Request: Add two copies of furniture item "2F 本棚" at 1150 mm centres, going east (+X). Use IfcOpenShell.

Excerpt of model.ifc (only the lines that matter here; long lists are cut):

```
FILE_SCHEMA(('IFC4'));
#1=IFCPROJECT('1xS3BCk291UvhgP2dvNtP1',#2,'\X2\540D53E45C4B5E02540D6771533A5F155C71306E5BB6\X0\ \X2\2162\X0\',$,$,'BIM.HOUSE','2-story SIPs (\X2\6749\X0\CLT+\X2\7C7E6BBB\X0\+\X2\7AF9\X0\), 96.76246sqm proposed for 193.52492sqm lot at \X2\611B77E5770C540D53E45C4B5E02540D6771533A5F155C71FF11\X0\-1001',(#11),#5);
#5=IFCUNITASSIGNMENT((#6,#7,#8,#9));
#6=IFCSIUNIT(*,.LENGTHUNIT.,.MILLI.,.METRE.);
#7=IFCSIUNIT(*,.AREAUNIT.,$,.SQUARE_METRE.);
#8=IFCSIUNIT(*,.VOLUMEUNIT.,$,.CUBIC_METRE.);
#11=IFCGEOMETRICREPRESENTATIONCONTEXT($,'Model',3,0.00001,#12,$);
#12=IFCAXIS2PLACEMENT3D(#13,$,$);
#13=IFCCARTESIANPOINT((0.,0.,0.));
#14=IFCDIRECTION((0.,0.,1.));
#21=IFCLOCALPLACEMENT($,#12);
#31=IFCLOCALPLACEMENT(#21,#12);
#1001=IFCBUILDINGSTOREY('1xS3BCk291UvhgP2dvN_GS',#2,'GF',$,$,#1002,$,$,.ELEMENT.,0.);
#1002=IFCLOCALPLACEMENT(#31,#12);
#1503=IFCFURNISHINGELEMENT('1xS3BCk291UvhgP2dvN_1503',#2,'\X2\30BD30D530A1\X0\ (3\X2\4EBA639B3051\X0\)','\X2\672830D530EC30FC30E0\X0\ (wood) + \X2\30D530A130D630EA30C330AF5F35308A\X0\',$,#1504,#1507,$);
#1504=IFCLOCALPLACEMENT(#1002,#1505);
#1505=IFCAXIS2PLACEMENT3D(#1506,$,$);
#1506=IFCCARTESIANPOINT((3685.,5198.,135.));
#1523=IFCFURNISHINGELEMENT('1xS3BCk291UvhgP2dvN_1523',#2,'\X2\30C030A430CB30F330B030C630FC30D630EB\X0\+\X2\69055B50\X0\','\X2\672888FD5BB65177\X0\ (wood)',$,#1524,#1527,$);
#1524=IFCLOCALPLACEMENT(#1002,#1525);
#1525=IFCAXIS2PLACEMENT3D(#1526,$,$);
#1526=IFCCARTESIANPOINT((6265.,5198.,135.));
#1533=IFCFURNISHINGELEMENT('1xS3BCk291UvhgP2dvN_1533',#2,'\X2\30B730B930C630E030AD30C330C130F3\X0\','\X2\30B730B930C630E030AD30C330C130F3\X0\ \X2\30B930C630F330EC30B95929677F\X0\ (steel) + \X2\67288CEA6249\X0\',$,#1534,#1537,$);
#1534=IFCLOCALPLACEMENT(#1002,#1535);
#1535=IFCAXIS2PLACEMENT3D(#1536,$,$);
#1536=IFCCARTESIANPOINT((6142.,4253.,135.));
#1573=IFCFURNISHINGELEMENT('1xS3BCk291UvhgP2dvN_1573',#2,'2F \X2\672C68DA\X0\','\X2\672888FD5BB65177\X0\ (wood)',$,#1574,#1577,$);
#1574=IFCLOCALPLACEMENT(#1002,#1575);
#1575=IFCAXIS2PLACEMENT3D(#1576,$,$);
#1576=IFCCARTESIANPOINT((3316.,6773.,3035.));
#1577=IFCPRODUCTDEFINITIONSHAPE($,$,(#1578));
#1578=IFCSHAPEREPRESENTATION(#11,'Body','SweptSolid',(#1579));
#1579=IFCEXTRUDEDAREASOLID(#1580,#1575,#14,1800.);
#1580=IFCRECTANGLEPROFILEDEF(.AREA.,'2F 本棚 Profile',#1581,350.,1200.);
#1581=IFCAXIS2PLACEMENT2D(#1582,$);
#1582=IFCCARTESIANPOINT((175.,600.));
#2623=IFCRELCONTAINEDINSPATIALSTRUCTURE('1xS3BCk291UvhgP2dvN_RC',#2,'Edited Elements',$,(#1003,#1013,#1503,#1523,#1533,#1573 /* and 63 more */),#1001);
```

```python
import numpy as np
import ifcopenshell
import ifcopenshell.api.geometry
import ifcopenshell.api.root
import ifcopenshell.util.element
import ifcopenshell.util.placement

model = ifcopenshell.open("model.ifc")


def reuse_history(source, copy):
    """copy_class also copies each property set's owner history, people and application; keep the originals."""
    for rel in copy.IsDefinedBy:
        if rel.is_a("IfcRelDefinesByProperties") and (history := rel.RelatingPropertyDefinition.OwnerHistory):
            rel.RelatingPropertyDefinition.OwnerHistory = source.OwnerHistory
            ifcopenshell.util.element.remove_deep2(model, history)


source = model.by_guid("1xS3BCk291UvhgP2dvN_1573")
base = ifcopenshell.util.placement.get_local_placement(source.ObjectPlacement)
step = np.array([1.0, 0.0, 0.0]) * 1150.0

for i in range(1, 3):
    copy = ifcopenshell.api.root.copy_class(model, product=source)
    copy.Representation = ifcopenshell.util.element.copy_deep(
        model, source.Representation, exclude=["IfcGeometricRepresentationContext", "IfcRepresentationMap"]
    )
    reuse_history(source, copy)
    matrix = base.copy()
    matrix[:3, 3] += i * step
    print("added at", matrix[:3, 3].round(3) + 0.0)
    ifcopenshell.api.geometry.edit_object_placement(model, product=copy, matrix=matrix, is_si=False)

model.write("model_rev.ifc")
```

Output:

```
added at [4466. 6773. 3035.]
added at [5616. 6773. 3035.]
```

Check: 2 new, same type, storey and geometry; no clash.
